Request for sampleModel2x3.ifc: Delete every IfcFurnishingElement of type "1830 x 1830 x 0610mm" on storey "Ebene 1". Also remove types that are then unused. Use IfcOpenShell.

First a look at what the model holds.

```python
import ifcopenshell
import ifcopenshell.util.element

model = ifcopenshell.open("sampleModel2x3.ifc")
print(model.schema)
storey = next(s for s in model.by_type("IfcBuildingStorey") if s.Name == "Ebene 1")
furniture = [e for e in ifcopenshell.util.element.get_decomposition(storey) if e.is_a("IfcFurnishingElement")]
seen = {}
for e in furniture:
    element_type = ifcopenshell.util.element.get_type(e)
    name = element_type.Name if element_type not in (None, e) else None
    seen[name] = seen.get(name, 0) + 1
for name, count in sorted(seen.items(), key=str):
    print(count, "x", name)
```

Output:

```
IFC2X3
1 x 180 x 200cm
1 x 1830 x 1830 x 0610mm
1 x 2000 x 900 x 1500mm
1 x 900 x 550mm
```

```python
import ifcopenshell
import ifcopenshell.api.root
import ifcopenshell.util.element

model = ifcopenshell.open("sampleModel2x3.ifc")

storey = next(s for s in model.by_type("IfcBuildingStorey") if s.Name == "Ebene 1")
furniture = [e for e in ifcopenshell.util.element.get_decomposition(storey) if e.is_a("IfcFurnishingElement")]
targets = [e for e in furniture if (t := ifcopenshell.util.element.get_type(e)) not in (None, e) and t.Name == "1830 x 1830 x 0610mm"]
types = {ifcopenshell.util.element.get_type(e) for e in targets} - {None, *targets}

for e in targets:
    ifcopenshell.api.root.remove_product(model, product=e)
print(len(targets), "removed")

unused = [t for t in types if not ifcopenshell.util.element.get_types(t)]
for t in unused:
    ifcopenshell.api.root.remove_product(model, product=t)
print(len(unused), "unused types removed")

model.write("sampleModel2x3_updated.ifc")
```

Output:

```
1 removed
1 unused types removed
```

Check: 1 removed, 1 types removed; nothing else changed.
